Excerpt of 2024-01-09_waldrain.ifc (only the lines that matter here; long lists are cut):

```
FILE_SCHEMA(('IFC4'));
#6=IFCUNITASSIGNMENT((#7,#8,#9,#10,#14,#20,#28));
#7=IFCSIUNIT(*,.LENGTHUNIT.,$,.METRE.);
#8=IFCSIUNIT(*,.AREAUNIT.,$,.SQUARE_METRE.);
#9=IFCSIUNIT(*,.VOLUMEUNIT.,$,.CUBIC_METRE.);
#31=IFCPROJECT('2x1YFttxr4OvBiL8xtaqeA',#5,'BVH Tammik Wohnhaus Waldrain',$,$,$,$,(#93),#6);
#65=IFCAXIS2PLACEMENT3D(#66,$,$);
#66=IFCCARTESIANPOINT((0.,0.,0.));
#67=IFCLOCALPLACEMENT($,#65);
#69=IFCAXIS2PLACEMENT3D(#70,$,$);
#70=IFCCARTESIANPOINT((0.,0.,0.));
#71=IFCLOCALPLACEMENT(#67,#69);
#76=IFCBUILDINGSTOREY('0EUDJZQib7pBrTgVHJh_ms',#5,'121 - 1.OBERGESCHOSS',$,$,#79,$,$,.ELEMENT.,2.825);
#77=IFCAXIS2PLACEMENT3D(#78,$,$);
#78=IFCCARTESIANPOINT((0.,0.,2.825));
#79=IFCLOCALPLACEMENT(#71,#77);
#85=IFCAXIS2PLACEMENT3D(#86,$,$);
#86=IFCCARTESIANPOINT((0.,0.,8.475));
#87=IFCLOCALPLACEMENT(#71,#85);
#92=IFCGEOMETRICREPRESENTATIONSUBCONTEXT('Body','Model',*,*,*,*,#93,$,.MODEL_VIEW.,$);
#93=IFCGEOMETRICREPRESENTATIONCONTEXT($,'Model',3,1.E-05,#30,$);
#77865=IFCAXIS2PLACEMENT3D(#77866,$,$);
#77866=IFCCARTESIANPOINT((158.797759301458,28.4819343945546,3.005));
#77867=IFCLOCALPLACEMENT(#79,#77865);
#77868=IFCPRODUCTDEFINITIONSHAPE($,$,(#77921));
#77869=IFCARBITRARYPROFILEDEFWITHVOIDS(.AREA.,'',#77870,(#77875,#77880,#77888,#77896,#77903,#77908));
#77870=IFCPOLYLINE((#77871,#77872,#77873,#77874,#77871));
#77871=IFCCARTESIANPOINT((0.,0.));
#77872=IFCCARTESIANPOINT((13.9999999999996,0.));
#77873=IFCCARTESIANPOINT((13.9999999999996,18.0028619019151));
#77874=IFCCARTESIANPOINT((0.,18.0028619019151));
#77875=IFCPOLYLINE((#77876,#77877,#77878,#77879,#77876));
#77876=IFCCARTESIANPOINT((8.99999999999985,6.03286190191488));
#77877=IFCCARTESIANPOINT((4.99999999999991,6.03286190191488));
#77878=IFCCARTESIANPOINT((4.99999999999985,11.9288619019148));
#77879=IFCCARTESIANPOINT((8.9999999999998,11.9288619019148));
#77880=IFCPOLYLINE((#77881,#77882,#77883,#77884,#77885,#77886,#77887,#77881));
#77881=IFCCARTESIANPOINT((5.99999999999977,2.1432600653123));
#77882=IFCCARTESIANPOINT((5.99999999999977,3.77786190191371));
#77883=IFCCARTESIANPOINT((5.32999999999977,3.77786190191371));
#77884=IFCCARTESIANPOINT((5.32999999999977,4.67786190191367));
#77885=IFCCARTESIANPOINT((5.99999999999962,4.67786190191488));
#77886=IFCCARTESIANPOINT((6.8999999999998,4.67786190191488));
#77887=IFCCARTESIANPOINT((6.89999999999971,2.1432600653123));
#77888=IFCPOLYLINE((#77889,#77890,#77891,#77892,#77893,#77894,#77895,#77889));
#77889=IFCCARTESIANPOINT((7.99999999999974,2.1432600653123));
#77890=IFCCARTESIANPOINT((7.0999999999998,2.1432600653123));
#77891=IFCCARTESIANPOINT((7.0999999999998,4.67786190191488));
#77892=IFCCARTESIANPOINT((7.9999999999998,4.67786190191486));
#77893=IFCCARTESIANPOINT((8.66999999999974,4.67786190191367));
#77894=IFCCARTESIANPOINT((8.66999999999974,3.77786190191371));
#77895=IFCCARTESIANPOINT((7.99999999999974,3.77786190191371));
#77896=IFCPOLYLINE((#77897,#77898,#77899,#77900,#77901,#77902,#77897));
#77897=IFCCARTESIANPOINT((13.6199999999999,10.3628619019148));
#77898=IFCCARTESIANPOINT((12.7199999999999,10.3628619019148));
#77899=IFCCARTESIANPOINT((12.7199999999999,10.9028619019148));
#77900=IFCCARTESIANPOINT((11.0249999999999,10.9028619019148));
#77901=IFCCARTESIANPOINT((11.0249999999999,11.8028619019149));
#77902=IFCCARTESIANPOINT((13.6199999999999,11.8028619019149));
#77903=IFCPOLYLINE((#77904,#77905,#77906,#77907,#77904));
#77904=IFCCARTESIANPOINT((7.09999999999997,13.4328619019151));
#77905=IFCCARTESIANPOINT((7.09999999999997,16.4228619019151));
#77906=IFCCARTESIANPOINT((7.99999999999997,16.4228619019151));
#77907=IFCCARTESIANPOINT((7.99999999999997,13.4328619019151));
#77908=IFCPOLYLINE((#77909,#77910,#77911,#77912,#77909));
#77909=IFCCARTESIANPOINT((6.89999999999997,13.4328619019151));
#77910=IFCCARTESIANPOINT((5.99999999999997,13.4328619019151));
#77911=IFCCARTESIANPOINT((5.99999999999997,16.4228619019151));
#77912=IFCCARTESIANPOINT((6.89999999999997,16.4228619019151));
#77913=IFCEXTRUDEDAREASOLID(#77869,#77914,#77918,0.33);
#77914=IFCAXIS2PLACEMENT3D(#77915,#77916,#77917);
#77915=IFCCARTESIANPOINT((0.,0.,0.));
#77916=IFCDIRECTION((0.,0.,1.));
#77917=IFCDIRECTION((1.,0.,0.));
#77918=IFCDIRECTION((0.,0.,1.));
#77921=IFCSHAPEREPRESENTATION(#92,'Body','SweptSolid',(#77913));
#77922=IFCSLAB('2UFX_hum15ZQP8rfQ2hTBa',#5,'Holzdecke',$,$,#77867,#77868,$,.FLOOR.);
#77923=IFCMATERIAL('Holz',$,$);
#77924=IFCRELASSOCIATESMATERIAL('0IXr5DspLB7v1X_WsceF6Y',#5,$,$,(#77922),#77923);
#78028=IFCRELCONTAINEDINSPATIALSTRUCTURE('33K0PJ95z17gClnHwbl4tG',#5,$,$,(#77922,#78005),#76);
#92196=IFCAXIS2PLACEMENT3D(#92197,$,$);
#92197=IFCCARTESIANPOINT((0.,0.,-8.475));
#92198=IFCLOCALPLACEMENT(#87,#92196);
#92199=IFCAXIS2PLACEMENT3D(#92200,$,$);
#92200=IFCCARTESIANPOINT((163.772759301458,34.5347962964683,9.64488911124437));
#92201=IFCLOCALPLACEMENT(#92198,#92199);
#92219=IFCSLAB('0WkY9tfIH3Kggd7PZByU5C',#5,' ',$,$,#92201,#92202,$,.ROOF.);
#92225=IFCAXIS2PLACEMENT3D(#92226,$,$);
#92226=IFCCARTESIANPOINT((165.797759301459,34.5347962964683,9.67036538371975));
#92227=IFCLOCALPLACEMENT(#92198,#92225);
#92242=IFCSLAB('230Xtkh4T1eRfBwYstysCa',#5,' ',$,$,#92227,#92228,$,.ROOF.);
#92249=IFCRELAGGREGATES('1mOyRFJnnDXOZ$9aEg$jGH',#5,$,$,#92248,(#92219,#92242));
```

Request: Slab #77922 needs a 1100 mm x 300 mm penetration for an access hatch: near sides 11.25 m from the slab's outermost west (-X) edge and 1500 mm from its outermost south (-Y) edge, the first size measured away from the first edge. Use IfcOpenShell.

```python
import numpy as np
import ifcopenshell
import ifcopenshell.api.feature
import ifcopenshell.api.geometry
import ifcopenshell.api.root
import ifcopenshell.geom
import ifcopenshell.util.placement
import ifcopenshell.util.representation
import ifcopenshell.util.shape
import ifcopenshell.util.unit

model = ifcopenshell.open("2024-01-09_waldrain.ifc")
unit_scale = ifcopenshell.util.unit.calculate_unit_scale(model)
settings = ifcopenshell.geom.settings()


def volume(element):
    """Net volume in cubic metres, openings subtracted."""
    shape = ifcopenshell.geom.create_shape(settings, element)
    return ifcopenshell.util.shape.get_volume(shape.geometry)


slab = model.by_guid("2UFX_hum15ZQP8rfQ2hTBa")
before = volume(slab)

# Extent in the slab's own axes, in metres. The edges named are its -X and -Y sides.
slab_shape = ifcopenshell.geom.create_shape(settings, slab)
vertices = ifcopenshell.util.shape.get_vertices(slab_shape.geometry)
x_min, y_min, bottom = vertices.min(axis=0)
top = vertices[:, 2].max()

opening = ifcopenshell.api.root.create_entity(model, ifc_class="IfcOpeningElement", name="Access hatch opening", predefined_type="OPENING")
context = ifcopenshell.util.representation.get_context(model, "Model", "Body", "MODEL_VIEW")
width, depth = 1.1, 0.3
outline = [(0.0, 0.0), (width, 0.0), (width, depth), (0.0, depth), (0.0, 0.0)]
# Overshoot both faces by 50 mm so the cut is clean.
shape = ifcopenshell.api.geometry.add_slab_representation(
    model, context=context, depth=top - bottom + 0.1, polyline=outline
)
ifcopenshell.api.geometry.assign_representation(model, product=opening, representation=shape)

matrix = ifcopenshell.util.placement.get_local_placement(slab.ObjectPlacement)
matrix[:, 3] = matrix @ np.append(np.array([x_min + 11.25, y_min + 1.5, bottom - 0.05]) / unit_scale, 1.0)
ifcopenshell.api.geometry.edit_object_placement(model, product=opening, matrix=matrix, is_si=False)
ifcopenshell.api.feature.add_feature(model, feature=opening, element=slab)

after = volume(slab)

print(f"slab volume {before:.3f} -> {after:.3f} m3")

model.write("2024-01-09_waldrain_edited.ifc")
```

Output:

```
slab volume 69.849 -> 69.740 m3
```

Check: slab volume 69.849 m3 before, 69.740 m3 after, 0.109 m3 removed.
